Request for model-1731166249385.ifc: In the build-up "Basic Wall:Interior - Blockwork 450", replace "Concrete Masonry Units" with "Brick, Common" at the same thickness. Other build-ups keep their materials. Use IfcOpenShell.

First a look at what the model holds.

```python
import ifcopenshell
import ifcopenshell.util.element

model = ifcopenshell.open("model-1731166249385.ifc")
print(model.schema)
for layer_set in model.by_type("IfcMaterialLayerSet"):
    if layer_set.LayerSetName == "Basic Wall:Interior - Blockwork 450":
        for layer in layer_set.MaterialLayers:
            print(layer.id(), layer.Material and layer.Material.Name, layer.LayerThickness, sep=" | ")
        print(len(ifcopenshell.util.element.get_elements_by_material(model, layer_set)), "elements and types use it")
print(sorted(m.Name for m in model.by_type("IfcMaterial") if m.Name)[:60])
```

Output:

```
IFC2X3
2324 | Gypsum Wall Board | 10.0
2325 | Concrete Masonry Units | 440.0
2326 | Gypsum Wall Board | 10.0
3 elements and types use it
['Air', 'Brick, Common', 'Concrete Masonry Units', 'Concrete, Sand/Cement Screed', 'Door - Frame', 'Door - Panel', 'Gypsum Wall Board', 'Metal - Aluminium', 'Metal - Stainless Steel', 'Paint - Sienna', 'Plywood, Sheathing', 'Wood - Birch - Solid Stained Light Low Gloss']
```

```python
import ifcopenshell
import ifcopenshell.api.material

model = ifcopenshell.open("model-1731166249385.ifc")

layer_set = next(s for s in model.by_type("IfcMaterialLayerSet") if s.LayerSetName == "Basic Wall:Interior - Blockwork 450")
layer = next(l for l in layer_set.MaterialLayers if l.Material and l.Material.Name == "Concrete Masonry Units")
material = next(m for m in model.by_type("IfcMaterial") if m.Name == "Brick, Common")

# Point this one layer at the other material; renaming the old one would change it everywhere.
ifcopenshell.api.material.edit_layer(model, layer=layer, attributes={}, material=material)

print([l.Material.Name if l.Material else None for l in layer_set.MaterialLayers])

model.write("model-1731166249385_v2.ifc")
```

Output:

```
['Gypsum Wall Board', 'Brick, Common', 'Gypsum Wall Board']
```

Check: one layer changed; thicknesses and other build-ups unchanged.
